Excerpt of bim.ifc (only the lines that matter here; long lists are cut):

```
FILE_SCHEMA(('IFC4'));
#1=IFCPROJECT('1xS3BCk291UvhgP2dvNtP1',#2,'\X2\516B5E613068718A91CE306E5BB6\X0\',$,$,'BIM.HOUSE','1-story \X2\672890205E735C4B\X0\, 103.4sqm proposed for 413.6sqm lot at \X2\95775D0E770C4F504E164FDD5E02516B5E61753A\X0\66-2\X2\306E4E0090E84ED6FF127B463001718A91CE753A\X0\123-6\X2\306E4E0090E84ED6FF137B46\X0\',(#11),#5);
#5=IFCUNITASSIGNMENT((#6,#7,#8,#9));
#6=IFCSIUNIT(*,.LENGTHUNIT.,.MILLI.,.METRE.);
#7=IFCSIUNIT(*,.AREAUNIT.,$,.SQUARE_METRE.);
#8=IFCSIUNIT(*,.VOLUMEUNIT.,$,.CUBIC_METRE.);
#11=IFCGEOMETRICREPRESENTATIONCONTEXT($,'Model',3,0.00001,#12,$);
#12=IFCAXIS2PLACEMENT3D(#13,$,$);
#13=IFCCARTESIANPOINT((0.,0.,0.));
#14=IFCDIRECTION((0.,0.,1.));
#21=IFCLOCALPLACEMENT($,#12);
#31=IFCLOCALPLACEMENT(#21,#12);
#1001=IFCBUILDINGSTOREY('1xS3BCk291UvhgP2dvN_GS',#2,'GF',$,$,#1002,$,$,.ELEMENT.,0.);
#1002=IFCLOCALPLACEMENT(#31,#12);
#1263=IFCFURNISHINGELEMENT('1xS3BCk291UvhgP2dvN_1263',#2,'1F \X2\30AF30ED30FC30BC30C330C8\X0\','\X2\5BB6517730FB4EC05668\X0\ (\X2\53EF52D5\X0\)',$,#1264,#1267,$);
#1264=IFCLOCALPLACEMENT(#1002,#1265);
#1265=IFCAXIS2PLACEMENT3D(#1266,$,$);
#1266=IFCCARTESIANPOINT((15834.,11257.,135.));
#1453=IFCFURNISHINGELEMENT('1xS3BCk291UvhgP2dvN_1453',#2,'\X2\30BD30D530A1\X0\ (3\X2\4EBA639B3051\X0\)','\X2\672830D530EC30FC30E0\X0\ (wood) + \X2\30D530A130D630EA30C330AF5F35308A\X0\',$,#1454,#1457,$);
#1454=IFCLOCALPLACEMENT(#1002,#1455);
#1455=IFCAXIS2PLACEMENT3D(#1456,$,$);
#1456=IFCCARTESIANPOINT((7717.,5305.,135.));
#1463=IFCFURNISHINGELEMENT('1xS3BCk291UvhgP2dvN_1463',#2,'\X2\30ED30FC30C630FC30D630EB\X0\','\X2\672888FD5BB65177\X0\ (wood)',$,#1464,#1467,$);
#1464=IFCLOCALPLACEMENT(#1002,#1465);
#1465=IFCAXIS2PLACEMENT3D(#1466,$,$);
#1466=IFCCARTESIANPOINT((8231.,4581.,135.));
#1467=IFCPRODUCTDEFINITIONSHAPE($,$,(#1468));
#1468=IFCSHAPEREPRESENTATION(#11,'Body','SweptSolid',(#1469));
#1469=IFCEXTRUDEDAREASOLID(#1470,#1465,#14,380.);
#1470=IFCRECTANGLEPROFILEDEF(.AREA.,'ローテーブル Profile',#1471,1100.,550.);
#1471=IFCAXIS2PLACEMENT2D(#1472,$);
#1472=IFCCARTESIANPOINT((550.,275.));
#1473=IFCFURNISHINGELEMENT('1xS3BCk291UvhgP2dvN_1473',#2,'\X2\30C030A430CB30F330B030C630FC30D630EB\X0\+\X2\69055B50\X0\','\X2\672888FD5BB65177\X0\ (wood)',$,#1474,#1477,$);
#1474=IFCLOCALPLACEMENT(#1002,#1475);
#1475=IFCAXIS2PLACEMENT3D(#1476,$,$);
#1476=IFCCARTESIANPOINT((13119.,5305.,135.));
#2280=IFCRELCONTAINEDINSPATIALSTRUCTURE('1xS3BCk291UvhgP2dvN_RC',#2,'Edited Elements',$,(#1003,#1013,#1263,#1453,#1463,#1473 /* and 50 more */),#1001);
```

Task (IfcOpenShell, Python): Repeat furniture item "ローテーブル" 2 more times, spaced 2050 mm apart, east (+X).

```python
import numpy as np
import ifcopenshell
import ifcopenshell.api.geometry
import ifcopenshell.api.root
import ifcopenshell.util.element
import ifcopenshell.util.placement

model = ifcopenshell.open("bim.ifc")


def reuse_history(source, copy):
    """copy_class also copies each property set's owner history, people and application; keep the originals."""
    for rel in copy.IsDefinedBy:
        if rel.is_a("IfcRelDefinesByProperties") and (history := rel.RelatingPropertyDefinition.OwnerHistory):
            rel.RelatingPropertyDefinition.OwnerHistory = source.OwnerHistory
            ifcopenshell.util.element.remove_deep2(model, history)


source = model.by_id(1463)
base = ifcopenshell.util.placement.get_local_placement(source.ObjectPlacement)
step = np.array([1.0, 0.0, 0.0]) * 2050.0

for i in range(1, 3):
    copy = ifcopenshell.api.root.copy_class(model, product=source)
    copy.Representation = ifcopenshell.util.element.copy_deep(
        model, source.Representation, exclude=["IfcGeometricRepresentationContext", "IfcRepresentationMap"]
    )
    reuse_history(source, copy)
    matrix = base.copy()
    matrix[:3, 3] += i * step
    print("added at", matrix[:3, 3].round(3) + 0.0)
    ifcopenshell.api.geometry.edit_object_placement(model, product=copy, matrix=matrix, is_si=False)

model.write("bim-out.ifc")
```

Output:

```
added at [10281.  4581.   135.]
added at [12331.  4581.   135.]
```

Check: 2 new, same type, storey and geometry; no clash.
